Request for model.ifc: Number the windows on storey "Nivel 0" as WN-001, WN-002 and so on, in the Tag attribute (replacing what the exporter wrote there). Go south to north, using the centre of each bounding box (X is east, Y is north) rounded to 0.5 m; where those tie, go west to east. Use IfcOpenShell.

First a look at what the model holds.

```python
import ifcopenshell
import ifcopenshell.util.element
import ifcopenshell.util.placement

model = ifcopenshell.open("model.ifc")
print(model.schema)
storey = next(s for s in model.by_type("IfcBuildingStorey") if s.Name == "Nivel 0")
windows = [e for e in ifcopenshell.util.element.get_decomposition(storey) if e.is_a("IfcWindow")]
for e in sorted(windows, key=lambda e: e.id()):
    origin = ifcopenshell.util.placement.get_local_placement(e.ObjectPlacement)[:3, 3]
    print(e.id(), e.Tag, e.Name, origin.round(2) + 0.0, sep=" | ")
```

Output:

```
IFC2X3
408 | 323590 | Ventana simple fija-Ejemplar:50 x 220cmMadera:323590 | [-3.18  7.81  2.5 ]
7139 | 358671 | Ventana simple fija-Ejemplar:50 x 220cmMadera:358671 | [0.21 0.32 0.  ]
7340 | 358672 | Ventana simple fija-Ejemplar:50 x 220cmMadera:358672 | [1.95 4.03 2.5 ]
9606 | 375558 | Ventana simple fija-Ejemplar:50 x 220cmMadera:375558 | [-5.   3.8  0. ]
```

```python
import ifcopenshell
import ifcopenshell.geom
import ifcopenshell.util.element
import ifcopenshell.util.shape

model = ifcopenshell.open("model.ifc")
settings = ifcopenshell.geom.settings()
settings.set("use-world-coords", True)


def centre(element):
    shape = ifcopenshell.geom.create_shape(settings, element)
    return ifcopenshell.util.shape.get_bbox_centroid(shape.geometry)


storey = next(s for s in model.by_type("IfcBuildingStorey") if s.Name == "Nivel 0")
windows = [e for e in ifcopenshell.util.element.get_decomposition(storey) if e.is_a("IfcWindow")]

# Insertion points can sit at a corner or the storey origin, so sort by the geometry (in metres).
centres = {e: centre(e) for e in windows}
windows.sort(key=lambda e: (round(centres[e][1] / 0.5), centres[e][0]))

for i, e in enumerate(windows, start=1):
    number = f"WN-0{i:02d}"
    e.Tag = number
    print(e.id(), number)

model.write("model_edited.ifc")
```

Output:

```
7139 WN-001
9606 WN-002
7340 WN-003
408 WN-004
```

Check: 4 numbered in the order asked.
